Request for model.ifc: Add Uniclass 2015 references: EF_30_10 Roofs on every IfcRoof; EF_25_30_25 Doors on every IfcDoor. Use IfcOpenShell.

First a look at what the model holds.

```python
import ifcopenshell

model = ifcopenshell.open("model.ifc")
print(model.schema)
print("classifications:", [c.Name for c in model.by_type("IfcClassification")])
for ifc_class in ("IfcDoor", "IfcRoof", "IfcStair", "IfcWall", "IfcWindow"):
    print(ifc_class, len(model.by_type(ifc_class)))
```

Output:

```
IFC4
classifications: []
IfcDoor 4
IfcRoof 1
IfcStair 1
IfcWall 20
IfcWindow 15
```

```python
import ifcopenshell
import ifcopenshell.api.classification

model = ifcopenshell.open("model.ifc")

system = ifcopenshell.api.classification.add_classification(model, classification="Uniclass 2015")

codes = {
    "IfcRoof": ("EF_30_10", "Roofs"),
    "IfcDoor": ("EF_25_30_25", "Doors"),
}
for ifc_class, (code, name) in codes.items():
    products = model.by_type(ifc_class)
    ifcopenshell.api.classification.add_reference(
        model, products=products, classification=system, identification=code, name=name
    )
    print(code, len(products))

model.write("model_edited.ifc")
```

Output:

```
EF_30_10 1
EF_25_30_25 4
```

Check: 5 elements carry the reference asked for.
